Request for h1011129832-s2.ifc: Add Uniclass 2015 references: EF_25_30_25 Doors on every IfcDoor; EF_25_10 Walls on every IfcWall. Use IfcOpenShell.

First a look at what the model holds.

```python
import ifcopenshell

model = ifcopenshell.open("h1011129832-s2.ifc")
print(model.schema)
print("classifications:", [c.Name for c in model.by_type("IfcClassification")])
for ifc_class in ("IfcDoor", "IfcRoof", "IfcStair", "IfcWall", "IfcWindow"):
    print(ifc_class, len(model.by_type(ifc_class)))
```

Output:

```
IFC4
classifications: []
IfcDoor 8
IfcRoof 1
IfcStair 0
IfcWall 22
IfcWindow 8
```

```python
import ifcopenshell
import ifcopenshell.api.classification

model = ifcopenshell.open("h1011129832-s2.ifc")

system = ifcopenshell.api.classification.add_classification(model, classification="Uniclass 2015")

codes = {
    "IfcDoor": ("EF_25_30_25", "Doors"),
    "IfcWall": ("EF_25_10", "Walls"),
}
for ifc_class, (code, name) in codes.items():
    products = model.by_type(ifc_class)
    ifcopenshell.api.classification.add_reference(
        model, products=products, classification=system, identification=code, name=name
    )
    print(code, len(products))

model.write("h1011129832-s2-out.ifc")
```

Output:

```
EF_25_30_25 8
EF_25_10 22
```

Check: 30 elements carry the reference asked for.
